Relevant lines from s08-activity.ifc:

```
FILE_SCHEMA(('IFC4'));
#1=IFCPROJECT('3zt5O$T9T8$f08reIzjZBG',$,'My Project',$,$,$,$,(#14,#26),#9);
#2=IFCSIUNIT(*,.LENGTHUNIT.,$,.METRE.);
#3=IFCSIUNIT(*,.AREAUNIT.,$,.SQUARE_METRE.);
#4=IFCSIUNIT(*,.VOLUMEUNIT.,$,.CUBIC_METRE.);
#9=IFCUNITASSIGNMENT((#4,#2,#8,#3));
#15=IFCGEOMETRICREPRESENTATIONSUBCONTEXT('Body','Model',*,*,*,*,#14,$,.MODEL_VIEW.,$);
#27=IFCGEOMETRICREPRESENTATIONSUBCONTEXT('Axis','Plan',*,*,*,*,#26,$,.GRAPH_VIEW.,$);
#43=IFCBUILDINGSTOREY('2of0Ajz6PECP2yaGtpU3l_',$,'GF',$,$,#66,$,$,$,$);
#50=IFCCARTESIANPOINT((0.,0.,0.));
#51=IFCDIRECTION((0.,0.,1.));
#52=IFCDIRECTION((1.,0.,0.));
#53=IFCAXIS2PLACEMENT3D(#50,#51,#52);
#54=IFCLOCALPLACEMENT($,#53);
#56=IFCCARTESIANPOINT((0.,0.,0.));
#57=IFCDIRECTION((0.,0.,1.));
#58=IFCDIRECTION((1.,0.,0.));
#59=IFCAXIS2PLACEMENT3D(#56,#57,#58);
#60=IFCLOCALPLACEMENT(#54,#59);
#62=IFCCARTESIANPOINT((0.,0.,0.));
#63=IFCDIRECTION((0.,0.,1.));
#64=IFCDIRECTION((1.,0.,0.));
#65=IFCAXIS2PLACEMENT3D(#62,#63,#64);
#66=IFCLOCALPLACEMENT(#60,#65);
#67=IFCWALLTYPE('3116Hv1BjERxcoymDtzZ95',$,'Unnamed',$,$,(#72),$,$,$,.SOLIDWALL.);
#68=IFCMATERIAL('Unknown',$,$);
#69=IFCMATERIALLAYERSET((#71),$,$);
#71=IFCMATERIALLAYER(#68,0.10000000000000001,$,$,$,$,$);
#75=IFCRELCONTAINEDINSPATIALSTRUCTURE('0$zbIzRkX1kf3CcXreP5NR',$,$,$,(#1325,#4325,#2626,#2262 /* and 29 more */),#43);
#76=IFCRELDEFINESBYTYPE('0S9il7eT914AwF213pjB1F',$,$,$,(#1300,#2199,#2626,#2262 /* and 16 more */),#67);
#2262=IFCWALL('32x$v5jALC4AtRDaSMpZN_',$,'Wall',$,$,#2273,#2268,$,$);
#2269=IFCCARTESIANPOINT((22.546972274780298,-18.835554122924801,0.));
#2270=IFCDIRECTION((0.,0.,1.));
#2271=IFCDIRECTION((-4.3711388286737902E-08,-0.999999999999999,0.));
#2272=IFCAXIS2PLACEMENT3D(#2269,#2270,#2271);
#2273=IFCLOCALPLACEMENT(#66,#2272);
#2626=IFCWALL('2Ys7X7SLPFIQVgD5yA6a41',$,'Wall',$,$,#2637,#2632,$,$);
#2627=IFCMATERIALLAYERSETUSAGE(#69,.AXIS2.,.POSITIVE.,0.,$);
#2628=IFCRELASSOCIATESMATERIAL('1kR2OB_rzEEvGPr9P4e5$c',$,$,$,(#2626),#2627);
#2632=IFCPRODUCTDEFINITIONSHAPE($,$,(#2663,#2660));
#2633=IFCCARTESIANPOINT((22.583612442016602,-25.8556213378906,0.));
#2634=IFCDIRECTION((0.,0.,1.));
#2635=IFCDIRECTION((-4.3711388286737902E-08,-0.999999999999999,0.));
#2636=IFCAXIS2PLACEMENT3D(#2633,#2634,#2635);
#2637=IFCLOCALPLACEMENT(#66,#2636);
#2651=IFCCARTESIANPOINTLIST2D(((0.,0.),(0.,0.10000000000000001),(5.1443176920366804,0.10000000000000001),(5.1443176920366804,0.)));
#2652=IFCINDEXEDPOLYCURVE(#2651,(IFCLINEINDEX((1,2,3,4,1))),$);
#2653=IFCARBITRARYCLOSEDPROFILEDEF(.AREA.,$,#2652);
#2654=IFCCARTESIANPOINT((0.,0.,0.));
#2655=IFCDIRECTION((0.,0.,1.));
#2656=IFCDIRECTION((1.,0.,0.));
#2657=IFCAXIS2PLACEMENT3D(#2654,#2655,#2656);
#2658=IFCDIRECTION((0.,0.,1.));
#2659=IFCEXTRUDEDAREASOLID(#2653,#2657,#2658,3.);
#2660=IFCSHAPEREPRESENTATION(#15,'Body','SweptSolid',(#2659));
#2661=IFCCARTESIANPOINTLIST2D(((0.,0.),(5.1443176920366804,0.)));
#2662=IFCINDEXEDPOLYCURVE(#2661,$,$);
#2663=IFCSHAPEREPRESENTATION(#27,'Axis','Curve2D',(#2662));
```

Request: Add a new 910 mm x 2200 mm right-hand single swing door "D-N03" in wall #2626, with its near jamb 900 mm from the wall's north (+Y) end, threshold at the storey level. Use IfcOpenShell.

```python
import numpy as np
import ifcopenshell
import ifcopenshell.api.feature
import ifcopenshell.api.geometry
import ifcopenshell.api.root
import ifcopenshell.api.spatial
import ifcopenshell.geom
import ifcopenshell.util.element
import ifcopenshell.util.placement
import ifcopenshell.util.representation
import ifcopenshell.util.shape
import ifcopenshell.util.unit

model = ifcopenshell.open("s08-activity.ifc")
unit_scale = ifcopenshell.util.unit.calculate_unit_scale(model)
settings = ifcopenshell.geom.settings()


def volume(element):
    """Net volume in cubic metres, openings subtracted."""
    shape = ifcopenshell.geom.create_shape(settings, element)
    return ifcopenshell.util.shape.get_volume(shape.geometry)


wall = model.by_id(2626)
storey = ifcopenshell.util.element.get_container(wall, ifc_class="IfcBuildingStorey")
context = ifcopenshell.util.representation.get_context(model, "Model", "Body", "MODEL_VIEW")
before = volume(wall)

width, height, from_end, sill = 0.91, 2.2, 0.9, 0.0  # metres

# The wall runs along its own X axis, and the end named is its -X end.
wall_shape = ifcopenshell.geom.create_shape(settings, wall)
x, y, z = ifcopenshell.util.shape.get_vertices(wall_shape.geometry).T
start = x.min() + from_end
face, thickness = float(y.min()), float(y.max() - y.min())
wall_matrix = ifcopenshell.util.placement.get_local_placement(wall.ObjectPlacement)
level = ifcopenshell.util.placement.get_local_placement(storey.ObjectPlacement)[2, 3]


def in_wall(x, y):
    """Placement at x, y metres in the wall's axes, at sill height."""
    matrix = wall_matrix.copy()
    matrix[:, 3] = wall_matrix @ np.array([x / unit_scale, y / unit_scale, 0.0, 1.0])
    matrix[2, 3] = level + sill / unit_scale
    return matrix


# Opening: a box that overshoots both wall faces by 50 mm.
opening = ifcopenshell.api.root.create_entity(model, ifc_class="IfcOpeningElement", predefined_type="OPENING")
box = ifcopenshell.api.geometry.add_wall_representation(
    model, context=context, length=width, height=height, thickness=thickness + 0.1
)
ifcopenshell.api.geometry.assign_representation(model, product=opening, representation=box)
ifcopenshell.api.geometry.edit_object_placement(model, product=opening, matrix=in_wall(start, face - 0.05), is_si=False)
ifcopenshell.api.feature.add_feature(model, feature=opening, element=wall)

door = ifcopenshell.api.root.create_entity(model, ifc_class="IfcDoor", name="D-N03", predefined_type="DOOR")
door.OverallWidth, door.OverallHeight = width / unit_scale, height / unit_scale
door.OperationType = "SINGLE_SWING_RIGHT"
body = ifcopenshell.api.geometry.add_door_representation(
    model,
    context=context,
    overall_width=door.OverallWidth,
    overall_height=door.OverallHeight,
    operation_type="SINGLE_SWING_RIGHT",
    lining_properties={"LiningDepth": thickness / unit_scale, "ThresholdDepth": thickness / unit_scale},
)
ifcopenshell.api.geometry.assign_representation(model, product=door, representation=body)
ifcopenshell.api.spatial.assign_container(model, products=[door], relating_structure=storey)
ifcopenshell.api.feature.add_filling(model, opening=opening, element=door)

# The lining spans the wall, so the door starts at the wall face.
ifcopenshell.api.geometry.edit_object_placement(model, product=door, matrix=in_wall(start, face), is_si=False)

after = volume(wall)

print(f"wall volume {before:.3f} -> {after:.3f} m3")

model.write("s08-activity_v2.ifc")
```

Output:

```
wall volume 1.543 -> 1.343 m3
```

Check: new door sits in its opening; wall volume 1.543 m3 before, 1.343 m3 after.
